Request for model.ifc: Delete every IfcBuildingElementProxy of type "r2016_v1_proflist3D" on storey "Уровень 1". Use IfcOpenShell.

First a look at what the model holds.

```python
import ifcopenshell
import ifcopenshell.util.element

model = ifcopenshell.open("model.ifc")
print(model.schema)
storey = next(s for s in model.by_type("IfcBuildingStorey") if s.Name == "Уровень 1")
proxies = [e for e in ifcopenshell.util.element.get_decomposition(storey) if e.is_a("IfcBuildingElementProxy")]
seen = {}
for e in proxies:
    element_type = ifcopenshell.util.element.get_type(e)
    name = element_type.Name if element_type not in (None, e) else None
    seen[name] = seen.get(name, 0) + 1
for name, count in sorted(seen.items(), key=str):
    print(count, "x", name)
```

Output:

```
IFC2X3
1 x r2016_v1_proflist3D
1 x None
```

```python
import ifcopenshell
import ifcopenshell.api.root
import ifcopenshell.util.element

model = ifcopenshell.open("model.ifc")

storey = next(s for s in model.by_type("IfcBuildingStorey") if s.Name == "Уровень 1")
proxies = [e for e in ifcopenshell.util.element.get_decomposition(storey) if e.is_a("IfcBuildingElementProxy")]
targets = [e for e in proxies if (t := ifcopenshell.util.element.get_type(e)) not in (None, e) and t.Name == "r2016_v1_proflist3D"]

for e in targets:
    ifcopenshell.api.root.remove_product(model, product=e)
print(len(targets), "removed")

model.write("model_v2.ifc")
```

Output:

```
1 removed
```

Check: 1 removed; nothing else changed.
